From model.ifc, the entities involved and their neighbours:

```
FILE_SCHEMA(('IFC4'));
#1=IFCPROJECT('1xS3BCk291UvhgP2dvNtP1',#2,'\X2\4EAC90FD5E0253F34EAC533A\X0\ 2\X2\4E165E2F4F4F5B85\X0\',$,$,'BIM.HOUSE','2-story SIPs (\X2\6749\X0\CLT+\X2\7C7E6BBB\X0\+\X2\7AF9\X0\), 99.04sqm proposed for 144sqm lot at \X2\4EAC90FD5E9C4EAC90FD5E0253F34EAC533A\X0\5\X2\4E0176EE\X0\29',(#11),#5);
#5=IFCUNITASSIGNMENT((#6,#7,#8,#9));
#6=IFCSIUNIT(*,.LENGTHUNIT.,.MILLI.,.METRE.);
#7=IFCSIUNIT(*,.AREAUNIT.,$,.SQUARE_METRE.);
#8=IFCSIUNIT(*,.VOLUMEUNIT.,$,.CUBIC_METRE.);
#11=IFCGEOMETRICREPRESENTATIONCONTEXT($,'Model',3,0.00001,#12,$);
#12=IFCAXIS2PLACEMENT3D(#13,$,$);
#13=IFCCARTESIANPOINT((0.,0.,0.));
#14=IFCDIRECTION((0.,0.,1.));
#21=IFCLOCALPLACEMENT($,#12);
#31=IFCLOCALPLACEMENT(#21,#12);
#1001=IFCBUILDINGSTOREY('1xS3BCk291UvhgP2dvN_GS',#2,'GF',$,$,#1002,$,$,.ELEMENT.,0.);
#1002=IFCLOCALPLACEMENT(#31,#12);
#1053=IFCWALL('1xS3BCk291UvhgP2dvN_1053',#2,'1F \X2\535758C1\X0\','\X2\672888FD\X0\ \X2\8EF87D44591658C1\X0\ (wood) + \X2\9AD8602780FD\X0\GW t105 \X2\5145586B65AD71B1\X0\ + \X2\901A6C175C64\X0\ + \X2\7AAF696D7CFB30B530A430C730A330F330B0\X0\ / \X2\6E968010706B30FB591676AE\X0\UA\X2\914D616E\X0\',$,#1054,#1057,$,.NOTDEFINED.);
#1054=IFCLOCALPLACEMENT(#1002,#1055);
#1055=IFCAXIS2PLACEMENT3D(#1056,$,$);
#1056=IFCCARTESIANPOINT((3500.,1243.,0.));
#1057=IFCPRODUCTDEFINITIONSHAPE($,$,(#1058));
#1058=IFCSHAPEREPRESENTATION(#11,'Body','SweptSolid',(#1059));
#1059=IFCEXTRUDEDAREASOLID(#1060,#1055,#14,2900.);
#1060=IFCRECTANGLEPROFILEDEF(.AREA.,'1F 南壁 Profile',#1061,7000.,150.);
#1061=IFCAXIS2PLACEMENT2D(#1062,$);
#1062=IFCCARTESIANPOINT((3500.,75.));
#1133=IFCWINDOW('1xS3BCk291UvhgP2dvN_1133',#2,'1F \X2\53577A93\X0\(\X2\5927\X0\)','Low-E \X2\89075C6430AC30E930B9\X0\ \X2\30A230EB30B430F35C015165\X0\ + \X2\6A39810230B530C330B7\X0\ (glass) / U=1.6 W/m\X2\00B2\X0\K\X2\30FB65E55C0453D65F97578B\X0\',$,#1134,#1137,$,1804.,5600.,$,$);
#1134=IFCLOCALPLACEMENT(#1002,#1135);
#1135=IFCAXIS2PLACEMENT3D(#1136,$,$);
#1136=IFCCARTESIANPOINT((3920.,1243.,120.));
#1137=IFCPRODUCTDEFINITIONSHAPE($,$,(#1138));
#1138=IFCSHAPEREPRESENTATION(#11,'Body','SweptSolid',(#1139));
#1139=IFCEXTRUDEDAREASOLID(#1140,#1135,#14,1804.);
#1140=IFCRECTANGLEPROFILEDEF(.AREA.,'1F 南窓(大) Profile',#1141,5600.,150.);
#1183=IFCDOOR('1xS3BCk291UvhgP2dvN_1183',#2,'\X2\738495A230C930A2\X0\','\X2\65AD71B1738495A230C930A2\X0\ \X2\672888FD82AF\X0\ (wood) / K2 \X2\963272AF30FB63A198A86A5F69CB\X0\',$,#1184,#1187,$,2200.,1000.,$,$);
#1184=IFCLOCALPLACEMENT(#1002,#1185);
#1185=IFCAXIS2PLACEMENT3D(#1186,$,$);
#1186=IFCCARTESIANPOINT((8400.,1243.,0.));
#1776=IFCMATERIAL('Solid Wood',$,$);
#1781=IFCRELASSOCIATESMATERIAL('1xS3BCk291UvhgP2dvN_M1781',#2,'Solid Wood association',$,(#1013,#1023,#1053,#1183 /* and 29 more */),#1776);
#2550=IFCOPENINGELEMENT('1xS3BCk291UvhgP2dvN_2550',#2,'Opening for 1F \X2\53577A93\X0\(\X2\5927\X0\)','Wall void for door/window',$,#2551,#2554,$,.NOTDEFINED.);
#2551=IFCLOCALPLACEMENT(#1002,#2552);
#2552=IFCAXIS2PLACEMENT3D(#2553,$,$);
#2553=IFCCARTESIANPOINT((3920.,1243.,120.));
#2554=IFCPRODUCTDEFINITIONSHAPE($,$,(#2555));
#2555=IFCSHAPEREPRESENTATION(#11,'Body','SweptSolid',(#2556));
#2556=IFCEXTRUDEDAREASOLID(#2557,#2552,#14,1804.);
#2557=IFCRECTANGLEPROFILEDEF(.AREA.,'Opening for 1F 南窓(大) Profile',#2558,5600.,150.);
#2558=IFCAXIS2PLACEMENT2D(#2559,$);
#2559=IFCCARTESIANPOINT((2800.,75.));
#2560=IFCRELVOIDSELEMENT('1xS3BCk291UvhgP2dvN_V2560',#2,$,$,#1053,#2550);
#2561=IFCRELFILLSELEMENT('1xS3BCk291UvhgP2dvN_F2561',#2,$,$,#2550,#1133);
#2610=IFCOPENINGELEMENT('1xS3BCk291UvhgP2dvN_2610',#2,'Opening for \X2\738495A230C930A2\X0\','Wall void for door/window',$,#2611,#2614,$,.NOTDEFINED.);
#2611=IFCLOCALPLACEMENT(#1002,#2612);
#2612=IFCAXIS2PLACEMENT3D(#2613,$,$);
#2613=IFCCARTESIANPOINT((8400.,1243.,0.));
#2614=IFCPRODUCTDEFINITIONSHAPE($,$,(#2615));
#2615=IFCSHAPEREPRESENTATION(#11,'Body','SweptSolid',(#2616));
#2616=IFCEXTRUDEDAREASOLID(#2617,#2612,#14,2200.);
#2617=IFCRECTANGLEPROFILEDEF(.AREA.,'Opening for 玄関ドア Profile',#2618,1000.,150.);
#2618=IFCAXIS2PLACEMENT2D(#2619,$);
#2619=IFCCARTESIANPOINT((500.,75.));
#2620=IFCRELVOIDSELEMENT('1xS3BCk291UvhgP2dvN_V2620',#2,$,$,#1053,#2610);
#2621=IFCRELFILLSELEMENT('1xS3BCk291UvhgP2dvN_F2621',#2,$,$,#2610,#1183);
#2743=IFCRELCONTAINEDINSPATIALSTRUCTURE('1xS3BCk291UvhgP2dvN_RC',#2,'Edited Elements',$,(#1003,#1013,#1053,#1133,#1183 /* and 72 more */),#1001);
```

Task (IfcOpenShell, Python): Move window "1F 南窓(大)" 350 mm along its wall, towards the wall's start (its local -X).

```python
import ifcopenshell
import ifcopenshell.api.geometry
import ifcopenshell.util.placement

model = ifcopenshell.open("model.ifc")

window = model.by_id(1133)
opening = window.FillsVoids[0].RelatingOpeningElement
wall = opening.VoidsElements[0].RelatingBuildingElement

wall_matrix = ifcopenshell.util.placement.get_local_placement(wall.ObjectPlacement)
shift = wall_matrix[:3, 0] * -350.0
before = ifcopenshell.util.placement.get_local_placement(window.ObjectPlacement)[:3, 3].copy()

# The window is not placed relative to its opening, so move both.
for product in (opening, window):
    matrix = ifcopenshell.util.placement.get_local_placement(product.ObjectPlacement)
    matrix[:3, 3] += shift
    ifcopenshell.api.geometry.edit_object_placement(model, product=product, matrix=matrix, is_si=False)

after = ifcopenshell.util.placement.get_local_placement(window.ObjectPlacement)[:3, 3]
print("window moved by", (after - before).round(3) + 0.0)

model.write("model-out.ifc")
```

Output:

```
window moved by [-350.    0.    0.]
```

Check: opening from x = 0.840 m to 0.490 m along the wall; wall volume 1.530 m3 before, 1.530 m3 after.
